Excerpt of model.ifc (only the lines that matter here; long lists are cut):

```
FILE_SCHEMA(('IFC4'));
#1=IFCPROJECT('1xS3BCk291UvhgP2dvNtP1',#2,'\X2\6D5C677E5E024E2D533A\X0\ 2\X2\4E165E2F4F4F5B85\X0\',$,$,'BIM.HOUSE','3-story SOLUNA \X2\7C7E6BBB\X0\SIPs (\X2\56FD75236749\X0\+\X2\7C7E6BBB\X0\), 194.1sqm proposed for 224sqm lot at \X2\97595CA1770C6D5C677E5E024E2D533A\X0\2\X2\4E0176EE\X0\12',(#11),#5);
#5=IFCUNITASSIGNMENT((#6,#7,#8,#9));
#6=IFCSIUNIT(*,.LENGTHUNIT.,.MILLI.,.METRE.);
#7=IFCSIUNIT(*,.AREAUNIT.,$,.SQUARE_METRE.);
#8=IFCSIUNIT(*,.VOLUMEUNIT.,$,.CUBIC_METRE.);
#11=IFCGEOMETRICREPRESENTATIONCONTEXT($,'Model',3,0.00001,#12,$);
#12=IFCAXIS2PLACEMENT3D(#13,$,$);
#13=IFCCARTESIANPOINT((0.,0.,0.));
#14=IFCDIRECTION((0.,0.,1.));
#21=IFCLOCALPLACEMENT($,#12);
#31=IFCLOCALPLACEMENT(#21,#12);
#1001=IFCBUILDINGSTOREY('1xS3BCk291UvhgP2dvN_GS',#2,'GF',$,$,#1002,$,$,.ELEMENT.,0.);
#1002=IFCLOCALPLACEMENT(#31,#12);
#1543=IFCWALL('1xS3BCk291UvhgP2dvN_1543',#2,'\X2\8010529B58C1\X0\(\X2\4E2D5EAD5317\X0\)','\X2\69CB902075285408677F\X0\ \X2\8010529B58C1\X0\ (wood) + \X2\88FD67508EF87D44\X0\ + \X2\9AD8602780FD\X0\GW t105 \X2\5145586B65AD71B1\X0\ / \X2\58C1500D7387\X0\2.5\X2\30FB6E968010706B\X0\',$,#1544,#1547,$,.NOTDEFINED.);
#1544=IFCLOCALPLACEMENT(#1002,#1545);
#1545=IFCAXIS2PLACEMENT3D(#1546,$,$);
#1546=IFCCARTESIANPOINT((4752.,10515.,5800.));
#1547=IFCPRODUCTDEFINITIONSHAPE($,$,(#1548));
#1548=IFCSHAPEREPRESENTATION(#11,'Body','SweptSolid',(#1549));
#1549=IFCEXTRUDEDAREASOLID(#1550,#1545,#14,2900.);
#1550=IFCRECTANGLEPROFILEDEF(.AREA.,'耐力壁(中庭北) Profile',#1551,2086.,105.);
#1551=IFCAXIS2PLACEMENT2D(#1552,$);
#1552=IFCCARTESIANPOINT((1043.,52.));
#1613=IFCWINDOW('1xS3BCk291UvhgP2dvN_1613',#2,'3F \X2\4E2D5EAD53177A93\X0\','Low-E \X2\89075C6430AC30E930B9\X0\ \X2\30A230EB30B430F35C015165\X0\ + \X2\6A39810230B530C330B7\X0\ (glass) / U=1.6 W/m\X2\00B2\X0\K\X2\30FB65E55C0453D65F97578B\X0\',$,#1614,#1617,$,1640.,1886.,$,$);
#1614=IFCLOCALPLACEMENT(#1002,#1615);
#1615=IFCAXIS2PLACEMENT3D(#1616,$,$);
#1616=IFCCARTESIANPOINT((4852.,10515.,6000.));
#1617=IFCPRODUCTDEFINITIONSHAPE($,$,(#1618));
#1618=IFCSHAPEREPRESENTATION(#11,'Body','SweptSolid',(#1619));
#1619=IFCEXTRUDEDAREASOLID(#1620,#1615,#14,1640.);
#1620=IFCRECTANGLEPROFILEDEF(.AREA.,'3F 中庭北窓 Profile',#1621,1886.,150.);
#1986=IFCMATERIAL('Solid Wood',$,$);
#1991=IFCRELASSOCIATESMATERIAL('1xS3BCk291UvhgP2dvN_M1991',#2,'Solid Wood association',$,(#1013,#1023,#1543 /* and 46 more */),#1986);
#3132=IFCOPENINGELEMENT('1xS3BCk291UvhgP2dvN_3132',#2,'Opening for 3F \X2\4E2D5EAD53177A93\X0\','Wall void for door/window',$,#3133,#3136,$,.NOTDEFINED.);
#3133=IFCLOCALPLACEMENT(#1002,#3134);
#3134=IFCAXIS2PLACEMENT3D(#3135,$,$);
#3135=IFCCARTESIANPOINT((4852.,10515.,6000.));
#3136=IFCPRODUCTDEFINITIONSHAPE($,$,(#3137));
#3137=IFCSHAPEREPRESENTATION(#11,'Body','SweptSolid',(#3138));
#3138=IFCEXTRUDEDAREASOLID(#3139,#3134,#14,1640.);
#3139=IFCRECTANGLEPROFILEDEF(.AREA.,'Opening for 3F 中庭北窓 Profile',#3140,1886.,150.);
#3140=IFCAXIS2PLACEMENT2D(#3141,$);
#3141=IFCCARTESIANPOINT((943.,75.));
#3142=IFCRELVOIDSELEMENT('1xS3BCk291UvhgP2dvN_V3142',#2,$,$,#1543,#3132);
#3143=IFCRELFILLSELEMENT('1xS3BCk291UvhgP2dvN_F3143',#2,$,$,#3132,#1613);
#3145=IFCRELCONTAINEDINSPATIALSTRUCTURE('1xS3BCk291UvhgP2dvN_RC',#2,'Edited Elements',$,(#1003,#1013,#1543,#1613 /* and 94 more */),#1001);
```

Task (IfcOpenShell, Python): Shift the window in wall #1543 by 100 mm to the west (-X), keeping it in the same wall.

```python
import ifcopenshell
import ifcopenshell.api.geometry
import ifcopenshell.util.placement
import ifcopenshell.util.unit

model = ifcopenshell.open("model.ifc")
unit_scale = ifcopenshell.util.unit.calculate_unit_scale(model)

window = model.by_guid("1xS3BCk291UvhgP2dvN_1613")
opening = window.FillsVoids[0].RelatingOpeningElement
wall = opening.VoidsElements[0].RelatingBuildingElement

wall_matrix = ifcopenshell.util.placement.get_local_placement(wall.ObjectPlacement)
shift = wall_matrix[:3, 0] * -0.1 / unit_scale
before = ifcopenshell.util.placement.get_local_placement(window.ObjectPlacement)[:3, 3].copy()

# The window is not placed relative to its opening, so move both.
for product in (opening, window):
    matrix = ifcopenshell.util.placement.get_local_placement(product.ObjectPlacement)
    matrix[:3, 3] += shift
    ifcopenshell.api.geometry.edit_object_placement(model, product=product, matrix=matrix, is_si=False)

after = ifcopenshell.util.placement.get_local_placement(window.ObjectPlacement)[:3, 3]
print("window moved by", (after - before).round(3) + 0.0)

model.write("model_edited.ifc")
```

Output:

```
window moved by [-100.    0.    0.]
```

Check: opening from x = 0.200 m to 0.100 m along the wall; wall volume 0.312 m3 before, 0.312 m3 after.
